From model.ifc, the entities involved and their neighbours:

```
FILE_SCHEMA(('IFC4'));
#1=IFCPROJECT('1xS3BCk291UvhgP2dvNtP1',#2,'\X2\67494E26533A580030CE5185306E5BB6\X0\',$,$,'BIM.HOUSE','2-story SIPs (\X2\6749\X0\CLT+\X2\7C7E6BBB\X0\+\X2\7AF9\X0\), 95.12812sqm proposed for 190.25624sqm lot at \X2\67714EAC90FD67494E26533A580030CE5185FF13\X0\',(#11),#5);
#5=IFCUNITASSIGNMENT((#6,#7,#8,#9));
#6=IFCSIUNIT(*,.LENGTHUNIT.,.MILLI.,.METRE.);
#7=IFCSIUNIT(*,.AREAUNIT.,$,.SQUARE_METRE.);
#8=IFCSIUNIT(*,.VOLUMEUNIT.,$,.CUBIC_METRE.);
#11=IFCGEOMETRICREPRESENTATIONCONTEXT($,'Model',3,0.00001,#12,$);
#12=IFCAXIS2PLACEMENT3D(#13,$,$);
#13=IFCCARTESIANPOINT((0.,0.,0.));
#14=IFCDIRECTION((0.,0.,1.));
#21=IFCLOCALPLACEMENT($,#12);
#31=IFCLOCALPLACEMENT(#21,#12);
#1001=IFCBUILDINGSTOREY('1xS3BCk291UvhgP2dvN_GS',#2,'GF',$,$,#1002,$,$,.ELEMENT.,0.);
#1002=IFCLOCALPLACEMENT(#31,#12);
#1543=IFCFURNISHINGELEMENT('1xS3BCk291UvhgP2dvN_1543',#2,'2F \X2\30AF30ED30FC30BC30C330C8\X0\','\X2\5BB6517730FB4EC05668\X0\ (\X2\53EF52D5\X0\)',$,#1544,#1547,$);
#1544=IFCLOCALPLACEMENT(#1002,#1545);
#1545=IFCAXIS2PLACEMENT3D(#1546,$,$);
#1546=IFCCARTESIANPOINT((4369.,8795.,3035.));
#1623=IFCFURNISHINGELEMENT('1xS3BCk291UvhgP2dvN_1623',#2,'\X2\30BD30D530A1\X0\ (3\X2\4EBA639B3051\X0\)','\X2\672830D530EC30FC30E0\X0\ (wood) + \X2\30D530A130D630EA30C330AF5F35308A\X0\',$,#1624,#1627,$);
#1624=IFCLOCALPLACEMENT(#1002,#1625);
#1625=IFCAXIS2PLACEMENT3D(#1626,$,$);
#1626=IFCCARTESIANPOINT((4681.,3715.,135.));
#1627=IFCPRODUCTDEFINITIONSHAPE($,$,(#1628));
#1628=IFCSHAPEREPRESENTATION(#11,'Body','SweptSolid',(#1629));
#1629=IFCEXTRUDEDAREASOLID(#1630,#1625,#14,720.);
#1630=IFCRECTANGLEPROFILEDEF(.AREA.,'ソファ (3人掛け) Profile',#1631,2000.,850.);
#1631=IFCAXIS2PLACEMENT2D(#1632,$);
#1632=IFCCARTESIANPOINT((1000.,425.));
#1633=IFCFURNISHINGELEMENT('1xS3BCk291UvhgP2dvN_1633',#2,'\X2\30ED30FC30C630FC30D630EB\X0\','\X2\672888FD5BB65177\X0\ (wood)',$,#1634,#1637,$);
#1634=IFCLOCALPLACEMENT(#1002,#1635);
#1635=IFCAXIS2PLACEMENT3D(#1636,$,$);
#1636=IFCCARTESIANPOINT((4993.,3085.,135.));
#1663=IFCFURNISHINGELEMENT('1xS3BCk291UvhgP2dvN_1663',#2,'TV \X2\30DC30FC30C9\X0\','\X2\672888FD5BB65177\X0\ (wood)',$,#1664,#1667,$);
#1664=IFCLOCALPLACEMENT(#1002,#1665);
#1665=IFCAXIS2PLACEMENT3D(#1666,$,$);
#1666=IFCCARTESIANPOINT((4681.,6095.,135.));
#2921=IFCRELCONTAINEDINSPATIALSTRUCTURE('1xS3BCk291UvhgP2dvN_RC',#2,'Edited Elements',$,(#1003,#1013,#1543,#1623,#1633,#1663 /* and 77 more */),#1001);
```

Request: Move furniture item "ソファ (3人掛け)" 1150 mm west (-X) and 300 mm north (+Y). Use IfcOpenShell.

```python
import ifcopenshell
import ifcopenshell.api.geometry
import ifcopenshell.util.placement
import ifcopenshell.util.unit

model = ifcopenshell.open("model.ifc")
unit_scale = ifcopenshell.util.unit.calculate_unit_scale(model)

item = model.by_guid("1xS3BCk291UvhgP2dvN_1623")
matrix = ifcopenshell.util.placement.get_local_placement(item.ObjectPlacement)
matrix[0, 3] -= 1.15 / unit_scale
matrix[1, 3] += 0.3 / unit_scale
ifcopenshell.api.geometry.edit_object_placement(model, product=item, matrix=matrix, is_si=False)

print(ifcopenshell.util.placement.get_local_placement(item.ObjectPlacement).round(3) + 0.0)

model.write("model_v2.ifc")
```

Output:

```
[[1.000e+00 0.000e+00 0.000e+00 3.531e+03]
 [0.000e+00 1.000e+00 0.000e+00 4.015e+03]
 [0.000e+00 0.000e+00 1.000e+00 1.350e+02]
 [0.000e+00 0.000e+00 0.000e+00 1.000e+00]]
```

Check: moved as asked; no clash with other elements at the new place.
